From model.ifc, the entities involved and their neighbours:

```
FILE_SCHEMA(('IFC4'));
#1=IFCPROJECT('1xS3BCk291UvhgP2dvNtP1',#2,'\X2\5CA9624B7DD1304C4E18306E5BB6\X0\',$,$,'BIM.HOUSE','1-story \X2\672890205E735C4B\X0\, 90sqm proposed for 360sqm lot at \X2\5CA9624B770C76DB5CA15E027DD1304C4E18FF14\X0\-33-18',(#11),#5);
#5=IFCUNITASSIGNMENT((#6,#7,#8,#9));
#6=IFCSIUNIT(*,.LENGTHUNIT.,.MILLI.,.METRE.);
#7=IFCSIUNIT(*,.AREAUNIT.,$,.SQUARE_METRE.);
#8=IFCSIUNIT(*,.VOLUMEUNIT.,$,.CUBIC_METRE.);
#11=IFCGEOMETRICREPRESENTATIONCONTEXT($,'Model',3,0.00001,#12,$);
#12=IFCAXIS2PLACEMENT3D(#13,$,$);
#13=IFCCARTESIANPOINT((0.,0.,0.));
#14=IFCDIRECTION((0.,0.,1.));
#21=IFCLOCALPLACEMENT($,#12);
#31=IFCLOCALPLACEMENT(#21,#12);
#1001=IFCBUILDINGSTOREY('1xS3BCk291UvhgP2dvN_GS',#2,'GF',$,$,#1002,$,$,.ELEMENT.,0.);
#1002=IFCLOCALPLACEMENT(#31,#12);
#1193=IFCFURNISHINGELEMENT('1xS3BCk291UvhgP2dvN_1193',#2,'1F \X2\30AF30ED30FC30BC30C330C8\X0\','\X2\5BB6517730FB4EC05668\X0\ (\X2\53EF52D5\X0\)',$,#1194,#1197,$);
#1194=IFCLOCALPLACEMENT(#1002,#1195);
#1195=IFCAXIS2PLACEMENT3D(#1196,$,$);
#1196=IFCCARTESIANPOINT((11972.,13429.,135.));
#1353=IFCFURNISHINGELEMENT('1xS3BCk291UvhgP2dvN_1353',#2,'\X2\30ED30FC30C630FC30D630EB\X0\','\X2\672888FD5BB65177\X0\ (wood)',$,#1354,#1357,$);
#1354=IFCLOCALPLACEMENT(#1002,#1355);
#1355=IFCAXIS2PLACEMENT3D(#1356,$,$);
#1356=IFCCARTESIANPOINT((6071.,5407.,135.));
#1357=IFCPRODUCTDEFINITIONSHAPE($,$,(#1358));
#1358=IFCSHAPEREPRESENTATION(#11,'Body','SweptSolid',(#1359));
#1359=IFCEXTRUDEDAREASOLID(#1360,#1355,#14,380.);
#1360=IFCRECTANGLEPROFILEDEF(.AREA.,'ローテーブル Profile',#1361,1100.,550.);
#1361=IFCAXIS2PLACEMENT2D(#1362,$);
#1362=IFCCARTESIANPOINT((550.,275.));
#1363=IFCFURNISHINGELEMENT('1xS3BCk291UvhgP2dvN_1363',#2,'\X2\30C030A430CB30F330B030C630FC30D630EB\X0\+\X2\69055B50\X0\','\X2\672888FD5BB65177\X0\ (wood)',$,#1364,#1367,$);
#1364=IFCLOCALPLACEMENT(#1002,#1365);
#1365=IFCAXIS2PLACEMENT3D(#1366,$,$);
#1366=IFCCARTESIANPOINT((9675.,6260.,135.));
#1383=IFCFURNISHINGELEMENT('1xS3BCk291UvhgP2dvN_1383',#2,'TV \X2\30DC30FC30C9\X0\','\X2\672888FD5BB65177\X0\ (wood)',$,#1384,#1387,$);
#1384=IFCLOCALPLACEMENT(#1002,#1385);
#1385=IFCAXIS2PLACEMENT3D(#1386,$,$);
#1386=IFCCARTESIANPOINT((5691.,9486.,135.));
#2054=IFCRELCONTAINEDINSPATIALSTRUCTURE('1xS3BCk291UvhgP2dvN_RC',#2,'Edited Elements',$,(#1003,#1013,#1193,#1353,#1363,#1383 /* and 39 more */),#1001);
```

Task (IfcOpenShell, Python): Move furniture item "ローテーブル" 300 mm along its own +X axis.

```python
import ifcopenshell
import ifcopenshell.api.geometry
import ifcopenshell.util.placement

model = ifcopenshell.open("model.ifc")

item = model.by_guid("1xS3BCk291UvhgP2dvN_1353")
matrix = ifcopenshell.util.placement.get_local_placement(item.ObjectPlacement)
matrix[:3, 3] += matrix[:3, 0] * 300.0
ifcopenshell.api.geometry.edit_object_placement(model, product=item, matrix=matrix, is_si=False)

print(ifcopenshell.util.placement.get_local_placement(item.ObjectPlacement).round(3) + 0.0)

model.write("model_rev.ifc")
```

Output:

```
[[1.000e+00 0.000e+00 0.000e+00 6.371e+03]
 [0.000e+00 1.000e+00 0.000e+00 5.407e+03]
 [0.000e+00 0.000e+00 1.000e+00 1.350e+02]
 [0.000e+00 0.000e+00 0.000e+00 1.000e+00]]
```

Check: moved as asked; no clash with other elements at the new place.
